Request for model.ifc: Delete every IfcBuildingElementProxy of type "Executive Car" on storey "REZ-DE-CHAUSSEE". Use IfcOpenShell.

First a look at what the model holds.

```python
import ifcopenshell
import ifcopenshell.util.element

model = ifcopenshell.open("model.ifc")
print(model.schema)
storey = next(s for s in model.by_type("IfcBuildingStorey") if s.Name == "REZ-DE-CHAUSSEE")
proxies = [e for e in ifcopenshell.util.element.get_decomposition(storey) if e.is_a("IfcBuildingElementProxy")]
seen = {}
for e in proxies:
    element_type = ifcopenshell.util.element.get_type(e)
    name = element_type.Name if element_type not in (None, e) else None
    seen[name] = seen.get(name, 0) + 1
for name, count in sorted(seen.items(), key=str):
    print(count, "x", name)
```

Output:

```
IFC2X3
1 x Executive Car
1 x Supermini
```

```python
import ifcopenshell
import ifcopenshell.api.root
import ifcopenshell.util.element

model = ifcopenshell.open("model.ifc")

storey = next(s for s in model.by_type("IfcBuildingStorey") if s.Name == "REZ-DE-CHAUSSEE")
proxies = [e for e in ifcopenshell.util.element.get_decomposition(storey) if e.is_a("IfcBuildingElementProxy")]
targets = [e for e in proxies if (t := ifcopenshell.util.element.get_type(e)) not in (None, e) and t.Name == "Executive Car"]

for e in targets:
    ifcopenshell.api.root.remove_product(model, product=e)
print(len(targets), "removed")

model.write("model_edited.ifc")
```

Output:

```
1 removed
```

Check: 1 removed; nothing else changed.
